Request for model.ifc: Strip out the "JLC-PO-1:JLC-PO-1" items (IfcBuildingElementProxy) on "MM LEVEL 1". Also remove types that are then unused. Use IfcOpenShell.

First a look at what the model holds.

```python
import ifcopenshell
import ifcopenshell.util.element

model = ifcopenshell.open("model.ifc")
print(model.schema)
storey = next(s for s in model.by_type("IfcBuildingStorey") if s.Name == "MM LEVEL 1")
proxies = [e for e in ifcopenshell.util.element.get_decomposition(storey) if e.is_a("IfcBuildingElementProxy")]
seen = {}
for e in proxies:
    element_type = ifcopenshell.util.element.get_type(e)
    name = element_type.Name if element_type not in (None, e) else None
    seen[name] = seen.get(name, 0) + 1
for name, count in sorted(seen.items(), key=str):
    print(count, "x", name)
```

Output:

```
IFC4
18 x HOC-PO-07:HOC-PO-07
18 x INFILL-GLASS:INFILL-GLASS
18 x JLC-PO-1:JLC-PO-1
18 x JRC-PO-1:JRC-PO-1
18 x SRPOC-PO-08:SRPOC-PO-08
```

```python
import ifcopenshell
import ifcopenshell.api.root
import ifcopenshell.util.element

model = ifcopenshell.open("model.ifc")

storey = next(s for s in model.by_type("IfcBuildingStorey") if s.Name == "MM LEVEL 1")
proxies = [e for e in ifcopenshell.util.element.get_decomposition(storey) if e.is_a("IfcBuildingElementProxy")]
targets = [e for e in proxies if (t := ifcopenshell.util.element.get_type(e)) not in (None, e) and t.Name == "JLC-PO-1:JLC-PO-1"]
types = {ifcopenshell.util.element.get_type(e) for e in targets} - {None, *targets}

for e in targets:
    ifcopenshell.api.root.remove_product(model, product=e)
print(len(targets), "removed")

unused = [t for t in types if not ifcopenshell.util.element.get_types(t)]
for t in unused:
    ifcopenshell.api.root.remove_product(model, product=t)
print(len(unused), "unused types removed")

model.write("model_rev.ifc")
```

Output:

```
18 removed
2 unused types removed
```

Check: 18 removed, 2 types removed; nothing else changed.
